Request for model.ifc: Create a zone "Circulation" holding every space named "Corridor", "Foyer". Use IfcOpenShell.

First a look at what the model holds.

```python
import ifcopenshell

model = ifcopenshell.open("model.ifc")
print(model.schema)
seen = {}
for space in model.by_type("IfcSpace"):
    seen[space.LongName] = seen.get(space.LongName, 0) + 1
for name, count in sorted(seen.items(), key=str):
    print(count, "x", name)
print("zones:", [z.Name for z in model.by_type("IfcZone")][:20])
```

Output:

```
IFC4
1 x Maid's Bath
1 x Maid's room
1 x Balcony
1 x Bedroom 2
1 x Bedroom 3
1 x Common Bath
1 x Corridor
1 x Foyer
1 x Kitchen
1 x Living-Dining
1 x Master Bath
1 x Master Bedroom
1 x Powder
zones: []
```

```python
import ifcopenshell
import ifcopenshell.api.group
import ifcopenshell.api.root

model = ifcopenshell.open("model.ifc")

names = {"Corridor", "Foyer"}
spaces = [s for s in model.by_type("IfcSpace") if s.LongName in names]

zone = ifcopenshell.api.root.create_entity(model, ifc_class="IfcZone", name="Circulation")
ifcopenshell.api.group.assign_group(model, products=spaces, group=zone)
print(len(spaces), "spaces in", zone.Name)

model.write("model_rev.ifc")
```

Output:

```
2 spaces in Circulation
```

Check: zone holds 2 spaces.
